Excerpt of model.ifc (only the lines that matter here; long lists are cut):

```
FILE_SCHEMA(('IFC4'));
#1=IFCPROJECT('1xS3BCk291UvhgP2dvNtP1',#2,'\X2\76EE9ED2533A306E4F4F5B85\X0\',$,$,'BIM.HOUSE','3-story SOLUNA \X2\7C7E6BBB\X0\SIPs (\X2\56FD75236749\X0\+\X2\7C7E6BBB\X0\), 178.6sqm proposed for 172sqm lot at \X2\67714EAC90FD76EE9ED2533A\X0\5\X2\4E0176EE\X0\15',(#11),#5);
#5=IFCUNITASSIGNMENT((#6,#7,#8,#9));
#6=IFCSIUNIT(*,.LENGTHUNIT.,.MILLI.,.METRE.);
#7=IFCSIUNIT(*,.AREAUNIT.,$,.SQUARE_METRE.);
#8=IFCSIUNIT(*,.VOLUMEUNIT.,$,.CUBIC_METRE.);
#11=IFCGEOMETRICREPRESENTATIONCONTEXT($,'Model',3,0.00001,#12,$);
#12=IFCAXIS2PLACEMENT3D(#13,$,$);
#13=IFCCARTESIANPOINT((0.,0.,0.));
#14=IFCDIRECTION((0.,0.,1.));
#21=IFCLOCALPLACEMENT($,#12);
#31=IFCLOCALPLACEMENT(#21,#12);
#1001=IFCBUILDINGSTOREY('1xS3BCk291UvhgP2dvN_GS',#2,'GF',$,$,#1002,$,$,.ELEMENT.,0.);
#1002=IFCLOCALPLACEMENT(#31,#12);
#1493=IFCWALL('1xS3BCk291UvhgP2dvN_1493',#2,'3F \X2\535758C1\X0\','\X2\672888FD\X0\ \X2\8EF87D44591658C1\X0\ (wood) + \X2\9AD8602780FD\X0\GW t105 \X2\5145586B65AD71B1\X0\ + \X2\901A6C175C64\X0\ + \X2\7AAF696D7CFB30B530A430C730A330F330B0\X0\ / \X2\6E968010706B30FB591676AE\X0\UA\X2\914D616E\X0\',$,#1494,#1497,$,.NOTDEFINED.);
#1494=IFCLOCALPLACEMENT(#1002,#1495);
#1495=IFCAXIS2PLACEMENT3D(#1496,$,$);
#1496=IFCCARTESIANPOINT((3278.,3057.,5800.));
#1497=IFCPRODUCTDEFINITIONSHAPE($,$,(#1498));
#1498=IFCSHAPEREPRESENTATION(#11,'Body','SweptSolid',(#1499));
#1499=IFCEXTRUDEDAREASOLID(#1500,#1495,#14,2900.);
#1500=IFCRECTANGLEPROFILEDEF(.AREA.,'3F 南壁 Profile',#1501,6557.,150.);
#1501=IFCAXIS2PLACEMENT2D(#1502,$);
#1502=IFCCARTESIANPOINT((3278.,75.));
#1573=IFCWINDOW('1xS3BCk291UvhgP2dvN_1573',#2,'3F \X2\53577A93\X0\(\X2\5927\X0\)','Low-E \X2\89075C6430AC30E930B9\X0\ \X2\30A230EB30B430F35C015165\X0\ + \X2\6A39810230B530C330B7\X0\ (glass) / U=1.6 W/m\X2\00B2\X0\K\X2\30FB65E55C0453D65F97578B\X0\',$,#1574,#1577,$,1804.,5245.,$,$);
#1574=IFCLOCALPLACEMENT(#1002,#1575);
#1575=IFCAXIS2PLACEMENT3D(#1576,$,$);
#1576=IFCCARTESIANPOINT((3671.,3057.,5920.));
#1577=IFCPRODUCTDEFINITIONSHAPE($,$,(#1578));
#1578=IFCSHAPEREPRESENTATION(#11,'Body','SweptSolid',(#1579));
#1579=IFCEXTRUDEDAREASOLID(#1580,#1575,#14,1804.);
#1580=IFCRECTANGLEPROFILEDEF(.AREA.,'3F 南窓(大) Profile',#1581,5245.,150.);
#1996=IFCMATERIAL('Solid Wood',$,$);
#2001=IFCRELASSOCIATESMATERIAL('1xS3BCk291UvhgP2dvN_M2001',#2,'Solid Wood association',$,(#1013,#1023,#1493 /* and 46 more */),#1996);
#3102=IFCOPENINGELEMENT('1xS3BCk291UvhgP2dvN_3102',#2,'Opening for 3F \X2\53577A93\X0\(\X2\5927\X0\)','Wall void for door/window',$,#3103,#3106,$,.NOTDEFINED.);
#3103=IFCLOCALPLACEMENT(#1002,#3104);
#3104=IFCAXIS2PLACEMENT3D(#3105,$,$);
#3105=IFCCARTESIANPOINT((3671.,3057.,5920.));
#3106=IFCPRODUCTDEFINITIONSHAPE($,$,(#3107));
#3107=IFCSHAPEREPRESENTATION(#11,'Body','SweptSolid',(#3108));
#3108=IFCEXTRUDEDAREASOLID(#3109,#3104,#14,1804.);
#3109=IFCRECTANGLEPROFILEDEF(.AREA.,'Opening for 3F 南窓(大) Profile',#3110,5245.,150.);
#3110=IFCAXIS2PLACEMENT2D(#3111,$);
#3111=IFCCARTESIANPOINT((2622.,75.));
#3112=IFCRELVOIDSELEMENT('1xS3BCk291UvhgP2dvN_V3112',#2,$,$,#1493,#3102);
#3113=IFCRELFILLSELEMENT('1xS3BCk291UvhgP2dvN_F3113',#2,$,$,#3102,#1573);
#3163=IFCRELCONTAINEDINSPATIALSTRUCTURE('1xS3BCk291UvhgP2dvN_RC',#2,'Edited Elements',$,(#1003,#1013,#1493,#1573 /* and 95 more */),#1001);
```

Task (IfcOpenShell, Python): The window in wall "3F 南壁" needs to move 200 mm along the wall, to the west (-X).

```python
import ifcopenshell
import ifcopenshell.api.geometry
import ifcopenshell.util.placement
import ifcopenshell.util.unit

model = ifcopenshell.open("model.ifc")
unit_scale = ifcopenshell.util.unit.calculate_unit_scale(model)

window = model.by_guid("1xS3BCk291UvhgP2dvN_1573")
opening = window.FillsVoids[0].RelatingOpeningElement
wall = opening.VoidsElements[0].RelatingBuildingElement

wall_matrix = ifcopenshell.util.placement.get_local_placement(wall.ObjectPlacement)
shift = wall_matrix[:3, 0] * -0.2 / unit_scale
before = ifcopenshell.util.placement.get_local_placement(window.ObjectPlacement)[:3, 3].copy()

# The window is not placed relative to its opening, so move both.
for product in (opening, window):
    matrix = ifcopenshell.util.placement.get_local_placement(product.ObjectPlacement)
    matrix[:3, 3] += shift
    ifcopenshell.api.geometry.edit_object_placement(model, product=product, matrix=matrix, is_si=False)

after = ifcopenshell.util.placement.get_local_placement(window.ObjectPlacement)[:3, 3]
print("window moved by", (after - before).round(3) + 0.0)

model.write("model-out.ifc")
```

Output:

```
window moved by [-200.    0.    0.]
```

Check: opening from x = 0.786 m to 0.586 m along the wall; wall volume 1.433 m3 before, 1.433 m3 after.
